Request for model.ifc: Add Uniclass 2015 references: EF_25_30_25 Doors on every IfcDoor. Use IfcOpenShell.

First a look at what the model holds.

```python
import ifcopenshell

model = ifcopenshell.open("model.ifc")
print(model.schema)
print("classifications:", [c.Name for c in model.by_type("IfcClassification")])
for ifc_class in ("IfcDoor", "IfcRoof", "IfcStair", "IfcWall", "IfcWindow"):
    print(ifc_class, len(model.by_type(ifc_class)))
```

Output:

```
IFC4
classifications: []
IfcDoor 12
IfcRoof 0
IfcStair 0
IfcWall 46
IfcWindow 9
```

```python
import ifcopenshell
import ifcopenshell.api.classification

model = ifcopenshell.open("model.ifc")

system = ifcopenshell.api.classification.add_classification(model, classification="Uniclass 2015")

codes = {
    "IfcDoor": ("EF_25_30_25", "Doors"),
}
for ifc_class, (code, name) in codes.items():
    products = model.by_type(ifc_class)
    ifcopenshell.api.classification.add_reference(
        model, products=products, classification=system, identification=code, name=name
    )
    print(code, len(products))

model.write("model_v2.ifc")
```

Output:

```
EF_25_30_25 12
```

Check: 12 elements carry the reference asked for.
